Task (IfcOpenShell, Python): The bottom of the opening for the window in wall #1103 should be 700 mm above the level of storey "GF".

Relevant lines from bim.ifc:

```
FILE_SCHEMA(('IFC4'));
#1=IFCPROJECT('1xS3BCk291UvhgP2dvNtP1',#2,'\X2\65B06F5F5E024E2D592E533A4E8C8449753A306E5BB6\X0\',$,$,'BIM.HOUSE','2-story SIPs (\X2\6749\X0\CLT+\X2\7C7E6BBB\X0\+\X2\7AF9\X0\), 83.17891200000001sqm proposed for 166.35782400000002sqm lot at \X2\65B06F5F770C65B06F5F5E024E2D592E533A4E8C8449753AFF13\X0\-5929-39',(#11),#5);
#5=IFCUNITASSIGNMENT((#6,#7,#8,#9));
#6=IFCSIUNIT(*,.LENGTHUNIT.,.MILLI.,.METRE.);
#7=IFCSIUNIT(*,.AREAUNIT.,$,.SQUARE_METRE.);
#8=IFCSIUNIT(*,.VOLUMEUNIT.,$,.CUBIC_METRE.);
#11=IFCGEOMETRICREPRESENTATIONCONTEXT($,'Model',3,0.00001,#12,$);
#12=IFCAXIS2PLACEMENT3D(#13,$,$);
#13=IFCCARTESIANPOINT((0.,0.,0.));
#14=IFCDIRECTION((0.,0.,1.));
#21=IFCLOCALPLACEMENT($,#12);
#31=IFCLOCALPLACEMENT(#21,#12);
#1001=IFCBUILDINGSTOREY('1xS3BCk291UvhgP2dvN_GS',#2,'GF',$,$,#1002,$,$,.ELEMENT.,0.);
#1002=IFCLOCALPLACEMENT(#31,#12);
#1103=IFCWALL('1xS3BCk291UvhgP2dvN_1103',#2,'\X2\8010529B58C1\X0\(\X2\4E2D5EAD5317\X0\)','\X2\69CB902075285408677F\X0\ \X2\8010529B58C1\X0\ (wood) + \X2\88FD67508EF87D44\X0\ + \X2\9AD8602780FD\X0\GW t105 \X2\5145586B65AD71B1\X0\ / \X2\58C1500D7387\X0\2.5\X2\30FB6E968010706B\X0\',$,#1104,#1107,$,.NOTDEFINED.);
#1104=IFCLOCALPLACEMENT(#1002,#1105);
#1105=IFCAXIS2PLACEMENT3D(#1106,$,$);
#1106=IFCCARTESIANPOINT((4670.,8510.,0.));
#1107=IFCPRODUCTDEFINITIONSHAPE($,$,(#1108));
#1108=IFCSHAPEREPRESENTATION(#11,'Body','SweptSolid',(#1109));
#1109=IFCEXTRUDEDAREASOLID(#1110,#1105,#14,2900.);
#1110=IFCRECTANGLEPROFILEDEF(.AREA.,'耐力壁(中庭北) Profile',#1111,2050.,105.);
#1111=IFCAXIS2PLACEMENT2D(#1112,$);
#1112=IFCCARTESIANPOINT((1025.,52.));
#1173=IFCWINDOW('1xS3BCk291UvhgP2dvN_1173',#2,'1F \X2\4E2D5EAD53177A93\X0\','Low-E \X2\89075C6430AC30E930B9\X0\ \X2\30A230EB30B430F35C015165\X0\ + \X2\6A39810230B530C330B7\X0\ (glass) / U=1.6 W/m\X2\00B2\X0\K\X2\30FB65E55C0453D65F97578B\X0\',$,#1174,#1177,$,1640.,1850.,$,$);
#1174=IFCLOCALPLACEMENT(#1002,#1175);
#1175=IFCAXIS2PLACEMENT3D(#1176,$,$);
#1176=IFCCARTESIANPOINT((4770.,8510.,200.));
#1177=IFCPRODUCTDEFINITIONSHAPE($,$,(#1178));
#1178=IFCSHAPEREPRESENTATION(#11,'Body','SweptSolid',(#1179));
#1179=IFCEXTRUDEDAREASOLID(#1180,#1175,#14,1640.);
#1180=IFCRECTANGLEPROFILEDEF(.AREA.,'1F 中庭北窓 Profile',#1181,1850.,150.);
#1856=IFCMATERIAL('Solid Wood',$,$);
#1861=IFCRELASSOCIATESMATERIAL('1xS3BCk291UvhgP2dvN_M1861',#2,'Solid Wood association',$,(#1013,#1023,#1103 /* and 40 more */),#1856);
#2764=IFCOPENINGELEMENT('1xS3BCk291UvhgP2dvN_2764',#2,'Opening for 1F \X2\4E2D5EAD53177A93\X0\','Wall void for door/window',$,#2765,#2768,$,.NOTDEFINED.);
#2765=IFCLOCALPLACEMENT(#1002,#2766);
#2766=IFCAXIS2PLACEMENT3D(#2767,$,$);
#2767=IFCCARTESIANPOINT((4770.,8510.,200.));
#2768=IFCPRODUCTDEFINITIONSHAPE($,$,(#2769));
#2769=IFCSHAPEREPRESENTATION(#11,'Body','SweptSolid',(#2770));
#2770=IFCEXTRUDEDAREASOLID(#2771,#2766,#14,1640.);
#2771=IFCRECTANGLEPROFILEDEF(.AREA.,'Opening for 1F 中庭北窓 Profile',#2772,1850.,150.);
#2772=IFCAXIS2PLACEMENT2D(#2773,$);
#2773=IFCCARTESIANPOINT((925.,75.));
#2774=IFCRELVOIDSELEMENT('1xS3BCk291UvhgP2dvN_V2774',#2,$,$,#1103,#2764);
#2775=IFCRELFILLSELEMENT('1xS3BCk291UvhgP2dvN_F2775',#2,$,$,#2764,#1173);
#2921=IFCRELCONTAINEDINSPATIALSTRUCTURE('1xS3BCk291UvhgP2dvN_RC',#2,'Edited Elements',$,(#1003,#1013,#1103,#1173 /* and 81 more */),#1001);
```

```python
import numpy as np
import ifcopenshell
import ifcopenshell.api.geometry
import ifcopenshell.geom
import ifcopenshell.util.element
import ifcopenshell.util.placement
import ifcopenshell.util.shape
import ifcopenshell.util.unit

model = ifcopenshell.open("bim.ifc")
unit_scale = ifcopenshell.util.unit.calculate_unit_scale(model)

window = model.by_guid("1xS3BCk291UvhgP2dvN_1173")
opening = window.FillsVoids[0].RelatingOpeningElement
storey = ifcopenshell.util.element.get_container(window, ifc_class="IfcBuildingStorey")
level = ifcopenshell.util.placement.get_local_placement(storey.ObjectPlacement)[2, 3]

# The opening's origin need not be at the sill, so measure its lowest point.
shape = ifcopenshell.geom.create_shape(ifcopenshell.geom.settings(), opening)
bottom = ifcopenshell.util.shape.get_shape_bottom_elevation(shape, shape.geometry) / unit_scale
dz = level + 0.7 / unit_scale - bottom

shift = np.array([0.0, 0.0, dz])
# The window is not placed relative to its opening, so move both.
for product in (opening, window):
    matrix = ifcopenshell.util.placement.get_local_placement(product.ObjectPlacement)
    matrix[:3, 3] += shift
    ifcopenshell.api.geometry.edit_object_placement(model, product=product, matrix=matrix, is_si=False)

print(f"moved by {dz * unit_scale:+.3f} m")

model.write("bim_edited.ifc")
```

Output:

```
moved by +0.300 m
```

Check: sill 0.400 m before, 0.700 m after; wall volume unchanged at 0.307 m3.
